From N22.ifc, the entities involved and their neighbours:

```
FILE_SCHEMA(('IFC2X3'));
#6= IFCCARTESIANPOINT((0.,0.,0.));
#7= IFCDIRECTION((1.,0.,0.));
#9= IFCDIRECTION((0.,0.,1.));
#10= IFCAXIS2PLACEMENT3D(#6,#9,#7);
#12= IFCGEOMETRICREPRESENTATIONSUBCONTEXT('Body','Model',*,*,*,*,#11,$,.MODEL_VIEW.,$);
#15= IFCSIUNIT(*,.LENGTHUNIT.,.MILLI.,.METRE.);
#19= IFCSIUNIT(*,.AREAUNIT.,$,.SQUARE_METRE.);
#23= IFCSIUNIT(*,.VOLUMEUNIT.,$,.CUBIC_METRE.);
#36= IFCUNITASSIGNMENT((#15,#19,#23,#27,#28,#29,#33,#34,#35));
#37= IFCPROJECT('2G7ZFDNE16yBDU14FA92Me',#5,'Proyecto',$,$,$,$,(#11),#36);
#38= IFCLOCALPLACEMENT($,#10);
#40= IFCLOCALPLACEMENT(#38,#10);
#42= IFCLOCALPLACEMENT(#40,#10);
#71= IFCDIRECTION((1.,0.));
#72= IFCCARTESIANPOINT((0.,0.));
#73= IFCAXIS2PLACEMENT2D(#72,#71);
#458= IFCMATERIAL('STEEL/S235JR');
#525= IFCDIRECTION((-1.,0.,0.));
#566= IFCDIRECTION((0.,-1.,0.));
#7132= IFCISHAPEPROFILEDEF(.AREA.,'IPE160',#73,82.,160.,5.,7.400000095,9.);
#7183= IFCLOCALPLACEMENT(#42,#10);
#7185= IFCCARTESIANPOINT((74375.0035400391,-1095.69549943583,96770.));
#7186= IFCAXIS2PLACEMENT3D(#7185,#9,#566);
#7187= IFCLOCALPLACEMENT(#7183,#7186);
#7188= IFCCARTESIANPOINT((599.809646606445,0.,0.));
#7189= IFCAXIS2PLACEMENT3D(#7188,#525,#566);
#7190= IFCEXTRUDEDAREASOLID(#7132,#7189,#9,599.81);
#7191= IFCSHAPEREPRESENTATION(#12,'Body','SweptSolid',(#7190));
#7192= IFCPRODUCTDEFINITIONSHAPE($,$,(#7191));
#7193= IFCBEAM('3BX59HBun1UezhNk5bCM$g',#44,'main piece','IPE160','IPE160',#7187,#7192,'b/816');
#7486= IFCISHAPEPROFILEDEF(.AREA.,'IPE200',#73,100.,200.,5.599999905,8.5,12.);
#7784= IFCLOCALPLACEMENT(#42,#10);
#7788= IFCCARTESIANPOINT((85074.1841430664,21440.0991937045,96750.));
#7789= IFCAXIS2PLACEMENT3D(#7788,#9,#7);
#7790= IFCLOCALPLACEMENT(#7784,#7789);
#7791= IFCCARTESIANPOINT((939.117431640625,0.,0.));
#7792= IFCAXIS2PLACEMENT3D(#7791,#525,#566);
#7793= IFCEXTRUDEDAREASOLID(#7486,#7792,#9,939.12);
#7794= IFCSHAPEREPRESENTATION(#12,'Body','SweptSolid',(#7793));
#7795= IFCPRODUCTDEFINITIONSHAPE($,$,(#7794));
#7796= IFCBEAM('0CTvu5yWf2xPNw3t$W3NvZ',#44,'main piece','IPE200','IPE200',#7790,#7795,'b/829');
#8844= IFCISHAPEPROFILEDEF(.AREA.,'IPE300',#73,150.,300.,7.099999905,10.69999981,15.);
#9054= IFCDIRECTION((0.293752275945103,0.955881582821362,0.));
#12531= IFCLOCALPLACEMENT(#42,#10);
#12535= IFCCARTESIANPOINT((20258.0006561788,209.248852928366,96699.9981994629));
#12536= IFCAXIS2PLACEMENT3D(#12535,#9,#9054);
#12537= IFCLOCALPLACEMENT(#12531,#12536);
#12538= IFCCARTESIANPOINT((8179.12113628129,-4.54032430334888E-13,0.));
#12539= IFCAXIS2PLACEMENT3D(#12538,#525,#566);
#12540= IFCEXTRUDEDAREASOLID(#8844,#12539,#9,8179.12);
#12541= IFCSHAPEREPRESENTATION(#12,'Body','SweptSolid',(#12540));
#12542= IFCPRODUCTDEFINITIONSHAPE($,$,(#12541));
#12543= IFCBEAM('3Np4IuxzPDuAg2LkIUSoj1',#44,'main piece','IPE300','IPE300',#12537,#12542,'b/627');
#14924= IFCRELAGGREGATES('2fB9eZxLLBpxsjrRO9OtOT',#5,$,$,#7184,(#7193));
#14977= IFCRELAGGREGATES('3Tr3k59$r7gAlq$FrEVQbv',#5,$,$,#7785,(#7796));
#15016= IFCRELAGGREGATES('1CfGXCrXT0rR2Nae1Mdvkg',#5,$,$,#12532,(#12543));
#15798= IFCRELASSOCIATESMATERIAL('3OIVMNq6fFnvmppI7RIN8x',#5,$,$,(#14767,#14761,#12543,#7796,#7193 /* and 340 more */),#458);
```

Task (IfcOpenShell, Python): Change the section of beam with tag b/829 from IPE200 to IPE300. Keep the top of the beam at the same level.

```python
import ifcopenshell
import ifcopenshell.util.element
import ifcopenshell.util.representation

model = ifcopenshell.open("N22.ifc")

member = model.by_guid("0CTvu5yWf2xPNw3t$W3NvZ")
source = next(p for p in model.by_type("IfcIShapeProfileDef") if p.ProfileName == "IPE300")

body = ifcopenshell.util.representation.get_representation(member, "Model", "Body")
solid = body.Items[0]
old_profile = solid.SweptArea

# Copy the section's sizes but keep this member's own profile position.
profile = ifcopenshell.util.element.copy(model, source)
# Profiles are centred, so shift by half the change in depth to hold the top.
shift = (old_profile.OverallDepth - profile.OverallDepth) / 2
x, y = old_profile.Position.Location.Coordinates
up = (0.0, 1.0)  # upwards, in the solid's own plane
location = model.createIfcCartesianPoint((x + up[0] * shift, y + up[1] * shift))
profile.Position = model.createIfcAxis2Placement2D(location, old_profile.Position.RefDirection)
solid.SweptArea = profile
if not model.get_total_inverses(old_profile):
    ifcopenshell.util.element.remove_deep2(model, old_profile)
member.Description = member.Description.replace("IPE200", "IPE300")
member.ObjectType = member.ObjectType.replace("IPE200", "IPE300")

print(solid.SweptArea)

model.write("N22_v2.ifc")
```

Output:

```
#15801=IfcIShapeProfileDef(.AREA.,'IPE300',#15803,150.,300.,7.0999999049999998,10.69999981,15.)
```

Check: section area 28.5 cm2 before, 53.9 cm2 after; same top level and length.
